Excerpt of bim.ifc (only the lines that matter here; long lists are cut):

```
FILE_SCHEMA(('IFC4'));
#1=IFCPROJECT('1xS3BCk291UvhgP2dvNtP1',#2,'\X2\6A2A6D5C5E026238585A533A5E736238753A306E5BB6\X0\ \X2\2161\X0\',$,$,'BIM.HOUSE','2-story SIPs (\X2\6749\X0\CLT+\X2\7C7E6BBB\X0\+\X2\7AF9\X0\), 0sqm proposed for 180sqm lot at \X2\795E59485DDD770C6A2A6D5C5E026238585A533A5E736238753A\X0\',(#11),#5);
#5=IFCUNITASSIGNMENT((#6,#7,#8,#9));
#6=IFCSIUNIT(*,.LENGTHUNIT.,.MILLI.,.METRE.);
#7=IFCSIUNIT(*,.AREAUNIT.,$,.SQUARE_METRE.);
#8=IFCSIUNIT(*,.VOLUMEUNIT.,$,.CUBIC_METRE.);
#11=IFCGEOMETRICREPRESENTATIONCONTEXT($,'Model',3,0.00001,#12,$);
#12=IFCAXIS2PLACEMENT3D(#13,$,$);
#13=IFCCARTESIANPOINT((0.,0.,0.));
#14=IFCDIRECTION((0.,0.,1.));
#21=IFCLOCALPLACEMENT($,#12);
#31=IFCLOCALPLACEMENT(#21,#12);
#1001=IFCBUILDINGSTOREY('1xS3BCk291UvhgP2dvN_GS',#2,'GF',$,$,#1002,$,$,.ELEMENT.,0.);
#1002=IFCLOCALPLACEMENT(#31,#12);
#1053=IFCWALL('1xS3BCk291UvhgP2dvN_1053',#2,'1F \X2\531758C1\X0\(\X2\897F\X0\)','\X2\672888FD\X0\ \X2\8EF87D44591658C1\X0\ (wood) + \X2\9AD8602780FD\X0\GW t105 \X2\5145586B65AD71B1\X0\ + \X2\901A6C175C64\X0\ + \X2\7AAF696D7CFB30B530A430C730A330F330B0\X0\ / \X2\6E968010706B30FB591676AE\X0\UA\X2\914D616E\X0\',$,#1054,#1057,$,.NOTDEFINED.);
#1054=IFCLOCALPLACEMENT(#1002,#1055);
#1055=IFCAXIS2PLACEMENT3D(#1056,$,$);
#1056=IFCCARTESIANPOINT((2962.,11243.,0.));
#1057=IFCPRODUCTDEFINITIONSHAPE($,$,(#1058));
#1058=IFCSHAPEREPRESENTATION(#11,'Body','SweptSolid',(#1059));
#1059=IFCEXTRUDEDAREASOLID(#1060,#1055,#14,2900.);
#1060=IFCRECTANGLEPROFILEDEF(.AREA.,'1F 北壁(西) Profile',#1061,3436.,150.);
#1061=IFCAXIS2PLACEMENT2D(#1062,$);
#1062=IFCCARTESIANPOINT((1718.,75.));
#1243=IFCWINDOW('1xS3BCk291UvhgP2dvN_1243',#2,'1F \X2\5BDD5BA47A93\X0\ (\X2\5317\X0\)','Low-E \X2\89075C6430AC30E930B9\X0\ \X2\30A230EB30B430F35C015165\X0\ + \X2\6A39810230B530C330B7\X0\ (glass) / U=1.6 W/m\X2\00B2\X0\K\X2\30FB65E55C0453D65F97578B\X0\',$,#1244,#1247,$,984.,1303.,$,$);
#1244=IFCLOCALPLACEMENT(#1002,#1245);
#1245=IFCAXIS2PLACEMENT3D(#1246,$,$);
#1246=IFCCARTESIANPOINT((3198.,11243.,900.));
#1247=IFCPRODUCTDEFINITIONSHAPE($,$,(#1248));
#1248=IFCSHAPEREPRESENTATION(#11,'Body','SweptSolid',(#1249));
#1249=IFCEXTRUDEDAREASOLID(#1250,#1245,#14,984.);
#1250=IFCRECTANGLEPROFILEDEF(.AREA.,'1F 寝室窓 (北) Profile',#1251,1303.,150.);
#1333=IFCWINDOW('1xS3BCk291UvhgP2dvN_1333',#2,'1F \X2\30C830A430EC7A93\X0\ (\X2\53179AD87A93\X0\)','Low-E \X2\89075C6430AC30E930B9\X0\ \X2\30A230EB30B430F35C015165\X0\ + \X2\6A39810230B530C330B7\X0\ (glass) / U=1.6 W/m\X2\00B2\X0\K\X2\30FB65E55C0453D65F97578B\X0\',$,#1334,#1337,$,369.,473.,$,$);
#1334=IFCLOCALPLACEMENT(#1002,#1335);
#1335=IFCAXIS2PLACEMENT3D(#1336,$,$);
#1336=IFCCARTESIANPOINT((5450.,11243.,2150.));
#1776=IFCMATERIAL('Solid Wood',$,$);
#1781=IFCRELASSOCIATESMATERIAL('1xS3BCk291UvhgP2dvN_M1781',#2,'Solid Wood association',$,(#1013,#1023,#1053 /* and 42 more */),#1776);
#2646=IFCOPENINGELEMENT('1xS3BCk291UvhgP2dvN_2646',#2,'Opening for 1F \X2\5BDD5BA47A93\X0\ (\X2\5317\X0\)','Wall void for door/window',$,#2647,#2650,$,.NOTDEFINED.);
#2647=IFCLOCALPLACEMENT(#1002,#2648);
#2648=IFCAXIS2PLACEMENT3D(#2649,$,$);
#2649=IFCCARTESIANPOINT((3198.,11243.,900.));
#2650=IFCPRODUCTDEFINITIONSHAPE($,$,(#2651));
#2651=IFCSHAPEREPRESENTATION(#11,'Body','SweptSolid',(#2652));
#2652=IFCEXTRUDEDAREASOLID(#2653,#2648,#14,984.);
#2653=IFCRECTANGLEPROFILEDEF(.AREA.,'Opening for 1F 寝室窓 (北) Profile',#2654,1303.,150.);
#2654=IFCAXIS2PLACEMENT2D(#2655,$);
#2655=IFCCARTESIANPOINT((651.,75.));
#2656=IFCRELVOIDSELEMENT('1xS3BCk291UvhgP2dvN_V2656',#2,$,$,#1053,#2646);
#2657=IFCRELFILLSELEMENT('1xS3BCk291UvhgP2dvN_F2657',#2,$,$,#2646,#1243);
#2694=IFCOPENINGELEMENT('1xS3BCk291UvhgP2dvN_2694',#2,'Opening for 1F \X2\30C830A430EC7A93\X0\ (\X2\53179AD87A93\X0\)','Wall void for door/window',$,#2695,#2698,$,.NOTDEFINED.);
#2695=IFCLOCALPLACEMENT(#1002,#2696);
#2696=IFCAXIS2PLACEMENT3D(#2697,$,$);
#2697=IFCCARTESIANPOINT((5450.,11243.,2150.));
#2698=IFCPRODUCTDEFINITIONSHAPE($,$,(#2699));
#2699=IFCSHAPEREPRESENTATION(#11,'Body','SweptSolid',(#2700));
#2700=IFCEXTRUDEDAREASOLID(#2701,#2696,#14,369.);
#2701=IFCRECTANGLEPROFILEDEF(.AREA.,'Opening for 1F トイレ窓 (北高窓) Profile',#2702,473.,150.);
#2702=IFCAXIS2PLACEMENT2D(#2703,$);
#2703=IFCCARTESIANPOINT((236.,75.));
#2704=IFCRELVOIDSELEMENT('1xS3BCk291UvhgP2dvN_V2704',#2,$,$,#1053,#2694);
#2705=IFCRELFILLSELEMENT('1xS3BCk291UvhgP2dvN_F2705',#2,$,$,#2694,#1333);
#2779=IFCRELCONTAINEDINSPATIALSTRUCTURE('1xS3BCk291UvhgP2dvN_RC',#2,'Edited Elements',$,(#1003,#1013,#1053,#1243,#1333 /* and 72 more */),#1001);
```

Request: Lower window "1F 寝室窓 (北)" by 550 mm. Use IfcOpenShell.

```python
import numpy as np
import ifcopenshell
import ifcopenshell.api.geometry
import ifcopenshell.util.placement
import ifcopenshell.util.unit

model = ifcopenshell.open("bim.ifc")
unit_scale = ifcopenshell.util.unit.calculate_unit_scale(model)

window = model.by_guid("1xS3BCk291UvhgP2dvN_1243")
opening = window.FillsVoids[0].RelatingOpeningElement
dz = -550.0

shift = np.array([0.0, 0.0, dz])
# The window is not placed relative to its opening, so move both.
for product in (opening, window):
    matrix = ifcopenshell.util.placement.get_local_placement(product.ObjectPlacement)
    matrix[:3, 3] += shift
    ifcopenshell.api.geometry.edit_object_placement(model, product=product, matrix=matrix, is_si=False)

print(f"moved by {dz * unit_scale:+.3f} m")

model.write("bim_rev.ifc")
```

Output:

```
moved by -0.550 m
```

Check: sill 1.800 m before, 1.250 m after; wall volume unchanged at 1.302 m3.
